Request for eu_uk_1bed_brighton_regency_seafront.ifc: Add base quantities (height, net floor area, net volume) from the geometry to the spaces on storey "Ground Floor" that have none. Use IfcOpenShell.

First a look at what the model holds.

```python
import ifcopenshell
import ifcopenshell.util.element
import ifcopenshell.util.unit

model = ifcopenshell.open("eu_uk_1bed_brighton_regency_seafront.ifc")
print(model.schema)
for unit_type in ("LENGTHUNIT", "AREAUNIT", "VOLUMEUNIT"):
    print(unit_type, ifcopenshell.util.unit.calculate_unit_scale(model, unit_type))
storey = next(s for s in model.by_type("IfcBuildingStorey") if s.Name == "Ground Floor")
spaces = [e for e in ifcopenshell.util.element.get_decomposition(storey) if e.is_a("IfcSpace")]
for e in sorted(spaces, key=lambda e: e.id()):
    print(e.id(), e.is_a(), e.Name, list(ifcopenshell.util.element.get_psets(e, qtos_only=True)), sep=" | ")
```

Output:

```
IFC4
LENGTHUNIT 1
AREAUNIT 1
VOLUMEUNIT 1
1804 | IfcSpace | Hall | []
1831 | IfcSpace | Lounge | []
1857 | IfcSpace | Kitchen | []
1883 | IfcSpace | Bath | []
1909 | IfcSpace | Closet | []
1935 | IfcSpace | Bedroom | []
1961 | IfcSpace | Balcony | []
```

```python
import ifcopenshell
import ifcopenshell.api.pset
import ifcopenshell.geom
import ifcopenshell.util.element
import ifcopenshell.util.shape
import ifcopenshell.util.unit

model = ifcopenshell.open("eu_uk_1bed_brighton_regency_seafront.ifc")
unit_scale = ifcopenshell.util.unit.calculate_unit_scale(model)
area_scale = ifcopenshell.util.unit.calculate_unit_scale(model, "AREAUNIT")
volume_scale = ifcopenshell.util.unit.calculate_unit_scale(model, "VOLUMEUNIT")
settings = ifcopenshell.geom.settings()

storey = next(s for s in model.by_type("IfcBuildingStorey") if s.Name == "Ground Floor")
spaces = [e for e in ifcopenshell.util.element.get_decomposition(storey) if e.is_a("IfcSpace")]

for e in sorted(spaces, key=lambda e: e.id()):
    if ifcopenshell.util.element.get_psets(e, qtos_only=True, should_inherit=False):
        continue
    # Geometry comes back in metres, in the element's own axes.
    shape = ifcopenshell.geom.create_shape(settings, e)
    values = {
        "Height": ifcopenshell.util.shape.get_z(shape.geometry) / unit_scale,
        "NetFloorArea": ifcopenshell.util.shape.get_footprint_area(shape.geometry) / area_scale,
        "NetVolume": ifcopenshell.util.shape.get_volume(shape.geometry) / volume_scale,
    }
    qto = ifcopenshell.api.pset.add_qto(model, product=e, name="Qto_SpaceBaseQuantities")
    ifcopenshell.api.pset.edit_qto(model, qto=qto, properties=values)
    print(e.id(), {k: round(v, 3) for k, v in values.items()})

model.write("eu_uk_1bed_brighton_regency_seafront-out.ifc")
```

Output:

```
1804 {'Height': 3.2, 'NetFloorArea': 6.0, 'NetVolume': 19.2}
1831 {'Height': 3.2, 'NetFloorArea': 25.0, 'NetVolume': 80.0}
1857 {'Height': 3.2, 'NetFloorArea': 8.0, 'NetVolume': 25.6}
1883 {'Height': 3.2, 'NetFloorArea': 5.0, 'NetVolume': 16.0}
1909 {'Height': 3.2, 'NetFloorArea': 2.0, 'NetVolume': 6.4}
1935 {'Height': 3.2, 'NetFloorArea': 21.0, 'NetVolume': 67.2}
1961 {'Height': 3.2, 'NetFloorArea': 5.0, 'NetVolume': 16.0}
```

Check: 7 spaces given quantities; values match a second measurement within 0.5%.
